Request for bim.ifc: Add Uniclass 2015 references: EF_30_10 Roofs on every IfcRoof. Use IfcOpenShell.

First a look at what the model holds.

```python
import ifcopenshell

model = ifcopenshell.open("bim.ifc")
print(model.schema)
print("classifications:", [c.Name for c in model.by_type("IfcClassification")])
for ifc_class in ("IfcDoor", "IfcRoof", "IfcStair", "IfcWall", "IfcWindow"):
    print(ifc_class, len(model.by_type(ifc_class)))
```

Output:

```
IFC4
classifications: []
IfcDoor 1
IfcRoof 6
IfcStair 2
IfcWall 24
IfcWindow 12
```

```python
import ifcopenshell
import ifcopenshell.api.classification

model = ifcopenshell.open("bim.ifc")

system = ifcopenshell.api.classification.add_classification(model, classification="Uniclass 2015")

codes = {
    "IfcRoof": ("EF_30_10", "Roofs"),
}
for ifc_class, (code, name) in codes.items():
    products = model.by_type(ifc_class)
    ifcopenshell.api.classification.add_reference(
        model, products=products, classification=system, identification=code, name=name
    )
    print(code, len(products))

model.write("bim_rev.ifc")
```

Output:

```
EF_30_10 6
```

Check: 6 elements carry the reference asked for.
